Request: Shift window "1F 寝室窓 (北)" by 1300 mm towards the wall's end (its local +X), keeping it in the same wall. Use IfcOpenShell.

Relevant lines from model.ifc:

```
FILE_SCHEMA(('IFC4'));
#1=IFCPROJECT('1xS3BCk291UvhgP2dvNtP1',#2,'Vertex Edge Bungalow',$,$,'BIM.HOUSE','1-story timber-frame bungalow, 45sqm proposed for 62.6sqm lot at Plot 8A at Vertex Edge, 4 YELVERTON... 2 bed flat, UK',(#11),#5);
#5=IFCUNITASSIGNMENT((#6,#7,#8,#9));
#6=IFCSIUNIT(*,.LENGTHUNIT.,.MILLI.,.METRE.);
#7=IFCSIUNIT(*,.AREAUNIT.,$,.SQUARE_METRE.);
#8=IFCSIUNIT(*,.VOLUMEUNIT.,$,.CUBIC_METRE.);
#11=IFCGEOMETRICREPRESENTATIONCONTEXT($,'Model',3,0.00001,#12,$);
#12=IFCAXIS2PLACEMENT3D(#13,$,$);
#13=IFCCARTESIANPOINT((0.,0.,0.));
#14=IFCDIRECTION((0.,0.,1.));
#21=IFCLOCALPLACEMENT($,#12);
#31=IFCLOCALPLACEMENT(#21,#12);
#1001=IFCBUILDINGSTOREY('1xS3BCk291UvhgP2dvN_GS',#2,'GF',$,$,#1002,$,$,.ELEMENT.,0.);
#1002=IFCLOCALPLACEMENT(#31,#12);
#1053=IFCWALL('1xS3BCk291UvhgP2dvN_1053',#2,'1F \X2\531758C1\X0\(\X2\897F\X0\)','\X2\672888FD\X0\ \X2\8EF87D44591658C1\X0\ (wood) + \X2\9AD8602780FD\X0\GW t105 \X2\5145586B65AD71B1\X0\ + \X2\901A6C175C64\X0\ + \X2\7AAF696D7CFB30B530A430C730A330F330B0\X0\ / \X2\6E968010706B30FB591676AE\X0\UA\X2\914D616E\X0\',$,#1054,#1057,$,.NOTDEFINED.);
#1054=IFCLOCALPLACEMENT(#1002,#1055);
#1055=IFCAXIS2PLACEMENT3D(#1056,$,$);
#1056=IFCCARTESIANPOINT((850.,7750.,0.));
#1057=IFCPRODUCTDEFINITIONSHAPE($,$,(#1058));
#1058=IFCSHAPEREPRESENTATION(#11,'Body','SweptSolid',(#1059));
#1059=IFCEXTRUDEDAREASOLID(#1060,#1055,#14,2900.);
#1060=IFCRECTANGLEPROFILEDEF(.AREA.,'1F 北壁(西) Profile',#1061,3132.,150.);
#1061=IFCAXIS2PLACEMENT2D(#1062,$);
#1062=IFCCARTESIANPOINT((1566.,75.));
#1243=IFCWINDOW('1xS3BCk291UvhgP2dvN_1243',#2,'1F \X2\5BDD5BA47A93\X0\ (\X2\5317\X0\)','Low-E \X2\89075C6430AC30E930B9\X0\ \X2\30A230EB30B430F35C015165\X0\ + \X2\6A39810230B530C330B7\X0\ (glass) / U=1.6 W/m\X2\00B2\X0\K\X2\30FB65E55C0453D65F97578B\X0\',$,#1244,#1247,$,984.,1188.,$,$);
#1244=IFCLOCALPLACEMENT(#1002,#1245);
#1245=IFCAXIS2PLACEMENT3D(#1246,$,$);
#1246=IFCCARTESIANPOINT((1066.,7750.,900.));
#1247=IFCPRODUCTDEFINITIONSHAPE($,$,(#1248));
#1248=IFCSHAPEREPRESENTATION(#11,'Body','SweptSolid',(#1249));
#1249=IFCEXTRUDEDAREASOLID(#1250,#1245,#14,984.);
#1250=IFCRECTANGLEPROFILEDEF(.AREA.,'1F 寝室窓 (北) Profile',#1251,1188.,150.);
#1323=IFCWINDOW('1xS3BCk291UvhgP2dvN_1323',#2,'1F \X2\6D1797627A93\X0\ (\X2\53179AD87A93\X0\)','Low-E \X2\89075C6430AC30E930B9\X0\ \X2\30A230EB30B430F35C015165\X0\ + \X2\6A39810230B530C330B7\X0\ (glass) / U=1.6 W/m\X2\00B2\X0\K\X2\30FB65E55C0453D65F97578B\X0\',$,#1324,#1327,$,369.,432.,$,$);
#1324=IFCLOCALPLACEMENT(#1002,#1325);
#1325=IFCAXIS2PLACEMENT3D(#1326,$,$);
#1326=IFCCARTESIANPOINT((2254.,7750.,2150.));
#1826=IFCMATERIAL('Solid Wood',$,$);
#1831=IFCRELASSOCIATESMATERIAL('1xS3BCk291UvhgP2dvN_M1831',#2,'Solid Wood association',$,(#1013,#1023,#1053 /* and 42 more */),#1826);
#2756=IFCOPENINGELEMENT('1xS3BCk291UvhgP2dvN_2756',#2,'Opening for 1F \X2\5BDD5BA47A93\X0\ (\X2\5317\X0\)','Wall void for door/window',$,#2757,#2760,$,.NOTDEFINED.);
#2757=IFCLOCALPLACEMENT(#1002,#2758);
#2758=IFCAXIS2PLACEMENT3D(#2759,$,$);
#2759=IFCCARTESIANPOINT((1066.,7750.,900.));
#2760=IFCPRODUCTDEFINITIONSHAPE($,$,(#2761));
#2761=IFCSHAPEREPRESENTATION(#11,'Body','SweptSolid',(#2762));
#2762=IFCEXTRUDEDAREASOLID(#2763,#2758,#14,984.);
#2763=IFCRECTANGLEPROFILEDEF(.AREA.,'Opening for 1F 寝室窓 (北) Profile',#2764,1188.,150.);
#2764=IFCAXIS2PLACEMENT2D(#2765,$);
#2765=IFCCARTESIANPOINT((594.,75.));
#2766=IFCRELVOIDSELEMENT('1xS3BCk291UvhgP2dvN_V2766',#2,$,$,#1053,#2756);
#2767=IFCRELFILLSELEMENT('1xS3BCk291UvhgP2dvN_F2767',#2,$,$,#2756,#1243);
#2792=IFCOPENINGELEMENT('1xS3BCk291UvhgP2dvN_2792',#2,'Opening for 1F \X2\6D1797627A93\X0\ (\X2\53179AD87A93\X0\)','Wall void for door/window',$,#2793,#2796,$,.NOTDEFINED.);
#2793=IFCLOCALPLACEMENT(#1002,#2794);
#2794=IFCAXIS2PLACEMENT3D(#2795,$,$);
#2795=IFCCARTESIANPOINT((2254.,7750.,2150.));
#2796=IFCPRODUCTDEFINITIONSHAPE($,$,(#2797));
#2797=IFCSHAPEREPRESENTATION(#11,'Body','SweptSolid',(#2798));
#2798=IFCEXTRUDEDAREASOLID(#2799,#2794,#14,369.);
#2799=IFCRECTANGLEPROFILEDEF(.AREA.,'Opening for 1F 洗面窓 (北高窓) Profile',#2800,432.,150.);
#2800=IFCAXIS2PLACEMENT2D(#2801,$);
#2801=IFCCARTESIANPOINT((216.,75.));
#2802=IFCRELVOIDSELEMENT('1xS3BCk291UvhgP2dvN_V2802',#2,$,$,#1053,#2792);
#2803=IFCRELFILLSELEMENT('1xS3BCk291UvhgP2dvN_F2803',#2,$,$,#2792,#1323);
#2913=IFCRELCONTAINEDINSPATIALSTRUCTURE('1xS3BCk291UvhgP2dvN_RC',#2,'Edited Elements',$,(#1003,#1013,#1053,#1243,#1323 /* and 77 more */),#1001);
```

```python
import ifcopenshell
import ifcopenshell.api.geometry
import ifcopenshell.util.placement
import ifcopenshell.util.unit

model = ifcopenshell.open("model.ifc")
unit_scale = ifcopenshell.util.unit.calculate_unit_scale(model)

window = model.by_guid("1xS3BCk291UvhgP2dvN_1243")
opening = window.FillsVoids[0].RelatingOpeningElement
wall = opening.VoidsElements[0].RelatingBuildingElement

wall_matrix = ifcopenshell.util.placement.get_local_placement(wall.ObjectPlacement)
shift = wall_matrix[:3, 0] * 1.3 / unit_scale
before = ifcopenshell.util.placement.get_local_placement(window.ObjectPlacement)[:3, 3].copy()

# The window is not placed relative to its opening, so move both.
for product in (opening, window):
    matrix = ifcopenshell.util.placement.get_local_placement(product.ObjectPlacement)
    matrix[:3, 3] += shift
    ifcopenshell.api.geometry.edit_object_placement(model, product=product, matrix=matrix, is_si=False)

after = ifcopenshell.util.placement.get_local_placement(window.ObjectPlacement)[:3, 3]
print("window moved by", (after - before).round(3) + 0.0)

model.write("model-out.ifc")
```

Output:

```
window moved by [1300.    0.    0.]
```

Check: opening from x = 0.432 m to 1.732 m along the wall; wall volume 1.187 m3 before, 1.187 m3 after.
